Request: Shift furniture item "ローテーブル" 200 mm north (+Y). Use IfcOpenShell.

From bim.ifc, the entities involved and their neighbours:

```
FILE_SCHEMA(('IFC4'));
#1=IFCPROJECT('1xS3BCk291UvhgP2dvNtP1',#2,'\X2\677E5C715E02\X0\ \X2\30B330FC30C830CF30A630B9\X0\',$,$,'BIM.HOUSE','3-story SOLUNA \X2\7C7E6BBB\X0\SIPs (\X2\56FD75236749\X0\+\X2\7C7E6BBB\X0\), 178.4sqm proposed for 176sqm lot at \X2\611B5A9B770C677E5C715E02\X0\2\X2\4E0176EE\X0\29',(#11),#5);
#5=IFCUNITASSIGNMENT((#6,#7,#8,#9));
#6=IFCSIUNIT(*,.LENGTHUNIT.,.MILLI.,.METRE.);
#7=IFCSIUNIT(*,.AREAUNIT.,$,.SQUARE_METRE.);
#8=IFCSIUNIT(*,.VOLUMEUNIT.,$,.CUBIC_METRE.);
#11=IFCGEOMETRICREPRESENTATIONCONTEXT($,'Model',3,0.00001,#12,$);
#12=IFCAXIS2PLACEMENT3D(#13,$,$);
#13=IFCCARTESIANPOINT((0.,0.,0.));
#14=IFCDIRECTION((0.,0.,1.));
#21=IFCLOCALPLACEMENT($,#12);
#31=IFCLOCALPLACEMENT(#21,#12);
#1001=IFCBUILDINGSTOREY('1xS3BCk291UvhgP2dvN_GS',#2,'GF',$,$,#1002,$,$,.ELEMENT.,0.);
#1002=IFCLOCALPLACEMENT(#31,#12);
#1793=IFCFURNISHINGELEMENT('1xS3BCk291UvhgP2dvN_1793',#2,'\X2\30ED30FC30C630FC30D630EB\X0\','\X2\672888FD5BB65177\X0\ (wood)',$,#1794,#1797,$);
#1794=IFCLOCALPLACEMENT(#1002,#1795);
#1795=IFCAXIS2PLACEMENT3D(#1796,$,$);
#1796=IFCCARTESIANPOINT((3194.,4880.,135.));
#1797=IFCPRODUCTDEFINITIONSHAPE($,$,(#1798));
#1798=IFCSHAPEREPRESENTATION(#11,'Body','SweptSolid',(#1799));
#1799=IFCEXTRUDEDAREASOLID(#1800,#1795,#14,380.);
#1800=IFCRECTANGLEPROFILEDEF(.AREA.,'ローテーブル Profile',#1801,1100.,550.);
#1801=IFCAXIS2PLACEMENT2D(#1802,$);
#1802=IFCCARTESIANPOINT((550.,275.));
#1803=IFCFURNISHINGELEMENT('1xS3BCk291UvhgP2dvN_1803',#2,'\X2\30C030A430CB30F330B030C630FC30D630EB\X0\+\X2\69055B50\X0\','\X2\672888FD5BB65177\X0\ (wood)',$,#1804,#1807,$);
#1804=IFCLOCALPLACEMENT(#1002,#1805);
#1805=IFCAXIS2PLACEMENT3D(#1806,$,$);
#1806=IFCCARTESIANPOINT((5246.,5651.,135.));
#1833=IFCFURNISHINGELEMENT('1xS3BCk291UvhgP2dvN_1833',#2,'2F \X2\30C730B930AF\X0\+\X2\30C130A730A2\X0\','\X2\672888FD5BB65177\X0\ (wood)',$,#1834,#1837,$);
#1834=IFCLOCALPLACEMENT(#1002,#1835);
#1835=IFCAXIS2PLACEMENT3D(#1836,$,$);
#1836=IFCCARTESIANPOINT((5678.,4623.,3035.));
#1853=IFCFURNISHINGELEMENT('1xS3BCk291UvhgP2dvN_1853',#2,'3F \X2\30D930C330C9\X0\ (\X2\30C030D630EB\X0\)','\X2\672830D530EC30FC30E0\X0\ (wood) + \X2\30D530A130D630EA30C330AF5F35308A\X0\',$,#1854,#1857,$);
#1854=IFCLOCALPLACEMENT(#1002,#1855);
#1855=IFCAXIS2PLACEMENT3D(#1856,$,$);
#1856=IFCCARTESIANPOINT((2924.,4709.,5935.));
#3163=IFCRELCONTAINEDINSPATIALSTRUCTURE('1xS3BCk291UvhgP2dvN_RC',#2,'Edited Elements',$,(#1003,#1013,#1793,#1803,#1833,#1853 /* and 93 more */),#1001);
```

```python
import ifcopenshell
import ifcopenshell.api.geometry
import ifcopenshell.util.placement

model = ifcopenshell.open("bim.ifc")

item = model.by_guid("1xS3BCk291UvhgP2dvN_1793")
matrix = ifcopenshell.util.placement.get_local_placement(item.ObjectPlacement)
matrix[1, 3] += 200.0
ifcopenshell.api.geometry.edit_object_placement(model, product=item, matrix=matrix, is_si=False)

print(ifcopenshell.util.placement.get_local_placement(item.ObjectPlacement).round(3) + 0.0)

model.write("bim_edited.ifc")
```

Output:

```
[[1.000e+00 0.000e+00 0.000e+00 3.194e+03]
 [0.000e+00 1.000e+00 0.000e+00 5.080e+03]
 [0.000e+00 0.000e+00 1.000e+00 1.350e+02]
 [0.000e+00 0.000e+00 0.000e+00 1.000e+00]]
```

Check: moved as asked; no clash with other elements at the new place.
